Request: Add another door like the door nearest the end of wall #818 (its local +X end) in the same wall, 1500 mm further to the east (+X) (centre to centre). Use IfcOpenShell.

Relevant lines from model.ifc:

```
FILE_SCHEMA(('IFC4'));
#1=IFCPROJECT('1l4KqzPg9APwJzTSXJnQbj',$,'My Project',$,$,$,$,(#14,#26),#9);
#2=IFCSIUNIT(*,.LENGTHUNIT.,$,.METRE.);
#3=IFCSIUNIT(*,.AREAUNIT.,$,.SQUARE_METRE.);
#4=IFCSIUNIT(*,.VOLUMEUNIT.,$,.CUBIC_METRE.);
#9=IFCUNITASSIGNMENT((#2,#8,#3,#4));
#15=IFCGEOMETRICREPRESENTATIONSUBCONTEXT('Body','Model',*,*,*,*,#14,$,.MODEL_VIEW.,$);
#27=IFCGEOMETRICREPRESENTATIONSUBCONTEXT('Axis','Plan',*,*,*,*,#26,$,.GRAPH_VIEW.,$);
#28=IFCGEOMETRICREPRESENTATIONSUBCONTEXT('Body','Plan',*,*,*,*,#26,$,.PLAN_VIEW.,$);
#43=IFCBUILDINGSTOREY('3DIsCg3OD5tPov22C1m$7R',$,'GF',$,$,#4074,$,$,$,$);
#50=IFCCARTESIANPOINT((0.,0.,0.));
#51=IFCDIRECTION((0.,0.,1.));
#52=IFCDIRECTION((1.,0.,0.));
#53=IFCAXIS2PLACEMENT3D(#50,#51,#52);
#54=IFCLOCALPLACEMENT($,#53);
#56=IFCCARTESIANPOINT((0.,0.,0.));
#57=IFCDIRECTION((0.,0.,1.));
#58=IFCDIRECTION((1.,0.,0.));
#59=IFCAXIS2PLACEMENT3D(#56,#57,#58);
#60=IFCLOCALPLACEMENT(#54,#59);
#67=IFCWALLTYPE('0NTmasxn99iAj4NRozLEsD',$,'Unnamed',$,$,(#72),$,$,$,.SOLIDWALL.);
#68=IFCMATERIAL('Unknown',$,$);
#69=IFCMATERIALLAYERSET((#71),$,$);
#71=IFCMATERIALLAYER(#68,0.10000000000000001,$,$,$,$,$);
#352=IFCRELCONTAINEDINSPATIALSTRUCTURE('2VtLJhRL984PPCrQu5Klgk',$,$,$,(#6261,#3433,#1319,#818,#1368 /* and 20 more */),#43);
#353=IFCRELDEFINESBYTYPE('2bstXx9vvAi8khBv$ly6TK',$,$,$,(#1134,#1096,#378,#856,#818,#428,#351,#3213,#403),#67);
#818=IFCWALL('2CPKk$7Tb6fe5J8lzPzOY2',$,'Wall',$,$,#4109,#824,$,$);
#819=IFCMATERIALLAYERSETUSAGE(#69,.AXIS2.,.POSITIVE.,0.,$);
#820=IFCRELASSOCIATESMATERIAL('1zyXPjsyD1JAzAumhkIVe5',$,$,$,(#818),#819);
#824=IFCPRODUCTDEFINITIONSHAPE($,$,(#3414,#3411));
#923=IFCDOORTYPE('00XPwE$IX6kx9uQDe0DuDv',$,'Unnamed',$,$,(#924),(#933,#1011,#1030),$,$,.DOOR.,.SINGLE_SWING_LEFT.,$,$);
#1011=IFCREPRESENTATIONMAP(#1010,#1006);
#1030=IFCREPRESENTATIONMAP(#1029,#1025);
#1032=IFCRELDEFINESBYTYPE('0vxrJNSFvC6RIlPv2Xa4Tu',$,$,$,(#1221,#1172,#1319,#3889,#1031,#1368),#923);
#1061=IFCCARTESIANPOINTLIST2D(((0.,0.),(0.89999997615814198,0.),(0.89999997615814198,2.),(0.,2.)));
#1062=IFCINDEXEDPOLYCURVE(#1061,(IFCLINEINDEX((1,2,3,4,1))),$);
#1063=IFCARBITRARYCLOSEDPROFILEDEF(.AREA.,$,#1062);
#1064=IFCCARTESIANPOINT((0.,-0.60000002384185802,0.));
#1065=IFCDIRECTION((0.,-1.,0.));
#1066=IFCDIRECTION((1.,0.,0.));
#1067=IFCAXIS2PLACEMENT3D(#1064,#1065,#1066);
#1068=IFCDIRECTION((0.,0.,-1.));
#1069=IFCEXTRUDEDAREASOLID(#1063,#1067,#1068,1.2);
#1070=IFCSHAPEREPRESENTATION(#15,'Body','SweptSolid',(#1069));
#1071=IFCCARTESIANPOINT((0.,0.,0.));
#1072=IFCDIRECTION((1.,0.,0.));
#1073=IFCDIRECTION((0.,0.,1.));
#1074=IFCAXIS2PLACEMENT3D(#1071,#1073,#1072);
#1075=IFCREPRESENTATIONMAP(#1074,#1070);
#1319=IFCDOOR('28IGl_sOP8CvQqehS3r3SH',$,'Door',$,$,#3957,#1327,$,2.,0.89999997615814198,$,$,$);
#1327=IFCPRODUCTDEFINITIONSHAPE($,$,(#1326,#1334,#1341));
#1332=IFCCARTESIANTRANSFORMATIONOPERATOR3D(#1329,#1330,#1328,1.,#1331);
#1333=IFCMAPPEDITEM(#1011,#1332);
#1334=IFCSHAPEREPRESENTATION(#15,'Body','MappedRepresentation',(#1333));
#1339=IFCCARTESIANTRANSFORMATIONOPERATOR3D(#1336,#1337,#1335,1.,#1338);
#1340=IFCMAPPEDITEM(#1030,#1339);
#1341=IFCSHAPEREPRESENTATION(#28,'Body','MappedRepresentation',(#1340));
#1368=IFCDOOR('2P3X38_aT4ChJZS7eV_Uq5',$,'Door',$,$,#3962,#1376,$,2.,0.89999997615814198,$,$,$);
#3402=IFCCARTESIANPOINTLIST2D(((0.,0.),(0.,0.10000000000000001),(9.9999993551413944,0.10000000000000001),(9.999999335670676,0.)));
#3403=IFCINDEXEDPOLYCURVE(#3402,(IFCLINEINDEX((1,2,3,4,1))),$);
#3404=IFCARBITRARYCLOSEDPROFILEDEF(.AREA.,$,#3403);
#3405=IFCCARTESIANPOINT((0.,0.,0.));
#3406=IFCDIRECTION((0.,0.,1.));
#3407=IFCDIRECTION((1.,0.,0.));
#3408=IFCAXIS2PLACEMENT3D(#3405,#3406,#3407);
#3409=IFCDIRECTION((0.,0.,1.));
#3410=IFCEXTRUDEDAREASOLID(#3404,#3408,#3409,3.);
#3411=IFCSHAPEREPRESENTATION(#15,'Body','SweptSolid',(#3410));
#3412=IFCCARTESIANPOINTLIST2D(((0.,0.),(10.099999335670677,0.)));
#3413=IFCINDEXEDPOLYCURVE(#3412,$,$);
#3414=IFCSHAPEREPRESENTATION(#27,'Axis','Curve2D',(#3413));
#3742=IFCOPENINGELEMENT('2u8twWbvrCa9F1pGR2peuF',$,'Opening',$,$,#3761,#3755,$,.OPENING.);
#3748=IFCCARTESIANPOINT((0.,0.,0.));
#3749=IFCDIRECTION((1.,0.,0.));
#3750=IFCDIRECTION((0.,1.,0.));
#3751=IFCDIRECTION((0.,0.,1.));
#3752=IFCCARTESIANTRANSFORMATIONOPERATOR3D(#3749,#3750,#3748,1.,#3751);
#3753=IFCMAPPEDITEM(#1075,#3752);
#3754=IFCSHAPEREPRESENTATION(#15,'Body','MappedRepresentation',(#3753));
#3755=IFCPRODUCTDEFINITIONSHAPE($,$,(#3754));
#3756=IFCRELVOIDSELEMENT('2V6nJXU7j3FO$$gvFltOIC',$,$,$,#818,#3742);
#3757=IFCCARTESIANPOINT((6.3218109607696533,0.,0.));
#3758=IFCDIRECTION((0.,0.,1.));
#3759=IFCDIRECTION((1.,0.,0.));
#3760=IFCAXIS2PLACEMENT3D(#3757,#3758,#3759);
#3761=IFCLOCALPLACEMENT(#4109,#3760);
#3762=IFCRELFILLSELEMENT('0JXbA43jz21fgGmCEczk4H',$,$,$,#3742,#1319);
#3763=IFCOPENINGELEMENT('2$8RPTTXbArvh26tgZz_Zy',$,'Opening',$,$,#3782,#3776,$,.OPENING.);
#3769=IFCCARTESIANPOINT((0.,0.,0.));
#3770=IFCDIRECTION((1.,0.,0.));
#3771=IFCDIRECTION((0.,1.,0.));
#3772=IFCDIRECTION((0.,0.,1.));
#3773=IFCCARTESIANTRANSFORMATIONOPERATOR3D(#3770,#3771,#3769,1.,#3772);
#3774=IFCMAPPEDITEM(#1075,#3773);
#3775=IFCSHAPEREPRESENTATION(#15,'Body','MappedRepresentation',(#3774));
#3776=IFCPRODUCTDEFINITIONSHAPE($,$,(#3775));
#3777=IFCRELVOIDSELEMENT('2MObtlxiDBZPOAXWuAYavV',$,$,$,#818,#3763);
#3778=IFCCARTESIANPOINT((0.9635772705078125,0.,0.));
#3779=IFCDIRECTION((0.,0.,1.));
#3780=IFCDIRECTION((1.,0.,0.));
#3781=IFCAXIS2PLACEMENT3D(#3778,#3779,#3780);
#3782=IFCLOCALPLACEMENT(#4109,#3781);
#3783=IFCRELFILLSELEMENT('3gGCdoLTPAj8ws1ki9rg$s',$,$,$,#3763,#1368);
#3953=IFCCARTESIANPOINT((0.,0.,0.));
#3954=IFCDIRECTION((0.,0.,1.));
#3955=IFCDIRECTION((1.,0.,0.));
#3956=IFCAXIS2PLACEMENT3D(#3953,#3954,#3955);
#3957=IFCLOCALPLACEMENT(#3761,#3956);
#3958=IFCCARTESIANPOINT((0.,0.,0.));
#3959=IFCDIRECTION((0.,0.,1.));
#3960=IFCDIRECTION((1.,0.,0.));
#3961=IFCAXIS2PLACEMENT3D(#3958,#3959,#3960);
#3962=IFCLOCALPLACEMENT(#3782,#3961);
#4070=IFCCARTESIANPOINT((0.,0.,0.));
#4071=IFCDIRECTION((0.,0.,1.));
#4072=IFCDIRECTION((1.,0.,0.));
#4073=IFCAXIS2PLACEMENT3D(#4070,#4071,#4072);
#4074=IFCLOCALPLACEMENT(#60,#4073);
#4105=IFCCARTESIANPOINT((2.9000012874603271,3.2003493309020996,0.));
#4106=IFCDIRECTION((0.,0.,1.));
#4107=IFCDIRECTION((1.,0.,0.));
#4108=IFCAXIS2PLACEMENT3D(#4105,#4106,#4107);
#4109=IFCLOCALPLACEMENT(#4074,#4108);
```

```python
import ifcopenshell
import ifcopenshell.api.feature
import ifcopenshell.api.geometry
import ifcopenshell.api.root
import ifcopenshell.geom
import ifcopenshell.util.element
import ifcopenshell.util.placement
import ifcopenshell.util.shape

model = ifcopenshell.open("model.ifc")
settings = ifcopenshell.geom.settings()


def volume(element):
    """Net volume in cubic metres, openings subtracted."""
    shape = ifcopenshell.geom.create_shape(settings, element)
    return ifcopenshell.util.shape.get_volume(shape.geometry)


door = model.by_guid("28IGl_sOP8CvQqehS3r3SH")
opening = door.FillsVoids[0].RelatingOpeningElement
wall = opening.VoidsElements[0].RelatingBuildingElement
before = volume(wall)
shift = ifcopenshell.util.placement.get_local_placement(wall.ObjectPlacement)[:3, 0] * 1.5

# copy_class copies the void relationship, type, container and properties, but no geometry.
new_opening = ifcopenshell.api.root.copy_class(model, product=opening)
new_opening.Representation = ifcopenshell.util.element.copy_deep(
    model, opening.Representation, exclude=["IfcGeometricRepresentationContext", "IfcRepresentationMap"]
)
new_door = ifcopenshell.api.root.copy_class(model, product=door)
new_door.Representation = ifcopenshell.util.element.copy_deep(
    model, door.Representation, exclude=["IfcGeometricRepresentationContext", "IfcRepresentationMap"]
)
ifcopenshell.api.feature.add_filling(model, opening=new_opening, element=new_door)

for old, new in ((opening, new_opening), (door, new_door)):
    matrix = ifcopenshell.util.placement.get_local_placement(old.ObjectPlacement)
    matrix[:3, 3] += shift
    ifcopenshell.api.geometry.edit_object_placement(model, product=new, matrix=matrix, is_si=False)

after = volume(wall)

print(f"wall volume {before:.3f} -> {after:.3f} m3")

model.write("model_rev.ifc")
```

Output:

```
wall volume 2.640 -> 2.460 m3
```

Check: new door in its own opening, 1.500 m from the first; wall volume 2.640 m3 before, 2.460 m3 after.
